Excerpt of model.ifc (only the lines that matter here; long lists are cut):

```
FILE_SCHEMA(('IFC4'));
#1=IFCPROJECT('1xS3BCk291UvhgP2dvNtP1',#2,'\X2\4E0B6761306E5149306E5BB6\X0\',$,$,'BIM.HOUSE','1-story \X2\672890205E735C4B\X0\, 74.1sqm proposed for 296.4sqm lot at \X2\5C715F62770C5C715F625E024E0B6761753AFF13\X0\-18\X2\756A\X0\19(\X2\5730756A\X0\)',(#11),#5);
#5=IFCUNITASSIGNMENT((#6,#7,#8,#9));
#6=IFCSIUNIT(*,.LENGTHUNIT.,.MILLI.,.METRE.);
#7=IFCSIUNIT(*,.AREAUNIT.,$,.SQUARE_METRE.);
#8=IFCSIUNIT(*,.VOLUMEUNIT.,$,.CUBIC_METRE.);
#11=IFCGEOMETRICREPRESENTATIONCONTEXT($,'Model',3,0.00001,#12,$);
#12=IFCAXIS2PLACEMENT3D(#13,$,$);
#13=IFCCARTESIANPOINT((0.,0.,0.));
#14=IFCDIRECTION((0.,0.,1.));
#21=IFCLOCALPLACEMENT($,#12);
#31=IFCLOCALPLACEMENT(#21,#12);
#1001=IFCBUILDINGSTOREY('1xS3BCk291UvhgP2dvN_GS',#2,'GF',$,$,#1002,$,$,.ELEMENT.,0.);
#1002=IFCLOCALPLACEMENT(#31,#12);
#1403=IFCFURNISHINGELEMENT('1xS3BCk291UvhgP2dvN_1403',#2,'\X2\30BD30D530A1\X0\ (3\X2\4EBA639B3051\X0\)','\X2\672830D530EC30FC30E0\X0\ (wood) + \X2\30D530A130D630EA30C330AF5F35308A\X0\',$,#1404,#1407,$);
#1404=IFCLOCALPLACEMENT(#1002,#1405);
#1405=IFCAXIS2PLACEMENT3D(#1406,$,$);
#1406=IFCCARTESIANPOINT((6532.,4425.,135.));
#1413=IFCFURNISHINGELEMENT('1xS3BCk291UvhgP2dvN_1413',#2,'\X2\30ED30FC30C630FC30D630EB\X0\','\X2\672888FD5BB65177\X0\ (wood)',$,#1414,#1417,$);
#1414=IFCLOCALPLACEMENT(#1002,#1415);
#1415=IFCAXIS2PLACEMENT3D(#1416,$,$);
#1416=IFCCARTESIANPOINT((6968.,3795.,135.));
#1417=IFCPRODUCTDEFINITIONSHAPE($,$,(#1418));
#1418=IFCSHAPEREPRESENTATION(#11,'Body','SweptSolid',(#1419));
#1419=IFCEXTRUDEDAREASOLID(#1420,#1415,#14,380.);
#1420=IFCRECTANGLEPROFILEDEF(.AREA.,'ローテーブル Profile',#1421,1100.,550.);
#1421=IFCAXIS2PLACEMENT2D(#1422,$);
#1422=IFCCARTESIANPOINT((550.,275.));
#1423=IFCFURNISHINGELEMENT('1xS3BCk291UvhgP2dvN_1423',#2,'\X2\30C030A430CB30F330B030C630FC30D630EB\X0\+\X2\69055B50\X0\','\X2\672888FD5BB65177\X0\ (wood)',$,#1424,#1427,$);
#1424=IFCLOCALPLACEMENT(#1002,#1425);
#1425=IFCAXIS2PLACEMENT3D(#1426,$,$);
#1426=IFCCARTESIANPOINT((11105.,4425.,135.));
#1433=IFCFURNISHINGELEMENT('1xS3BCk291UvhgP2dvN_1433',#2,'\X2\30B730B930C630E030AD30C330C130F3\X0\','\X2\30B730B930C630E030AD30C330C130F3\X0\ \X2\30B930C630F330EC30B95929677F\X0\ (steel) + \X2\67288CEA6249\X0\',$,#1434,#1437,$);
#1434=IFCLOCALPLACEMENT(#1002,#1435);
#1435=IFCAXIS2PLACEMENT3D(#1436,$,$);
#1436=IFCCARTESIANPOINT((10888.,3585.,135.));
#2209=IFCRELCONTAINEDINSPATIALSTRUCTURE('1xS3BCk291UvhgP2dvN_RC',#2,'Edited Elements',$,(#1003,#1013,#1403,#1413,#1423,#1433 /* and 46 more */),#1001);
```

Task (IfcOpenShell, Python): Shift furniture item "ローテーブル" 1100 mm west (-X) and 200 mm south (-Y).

```python
import ifcopenshell
import ifcopenshell.api.geometry
import ifcopenshell.util.placement
import ifcopenshell.util.unit

model = ifcopenshell.open("model.ifc")
unit_scale = ifcopenshell.util.unit.calculate_unit_scale(model)

item = model.by_id(1413)
matrix = ifcopenshell.util.placement.get_local_placement(item.ObjectPlacement)
matrix[0, 3] -= 1.1 / unit_scale
matrix[1, 3] -= 0.2 / unit_scale
ifcopenshell.api.geometry.edit_object_placement(model, product=item, matrix=matrix, is_si=False)

print(ifcopenshell.util.placement.get_local_placement(item.ObjectPlacement).round(3) + 0.0)

model.write("model_edited.ifc")
```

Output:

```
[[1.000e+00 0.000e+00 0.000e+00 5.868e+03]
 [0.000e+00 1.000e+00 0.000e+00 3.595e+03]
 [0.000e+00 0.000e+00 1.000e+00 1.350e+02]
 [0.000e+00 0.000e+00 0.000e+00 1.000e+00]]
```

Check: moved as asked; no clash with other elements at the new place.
